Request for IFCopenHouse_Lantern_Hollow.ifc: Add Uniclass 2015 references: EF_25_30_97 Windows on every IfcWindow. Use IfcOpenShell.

First a look at what the model holds.

```python
import ifcopenshell

model = ifcopenshell.open("IFCopenHouse_Lantern_Hollow.ifc")
print(model.schema)
print("classifications:", [c.Name for c in model.by_type("IfcClassification")])
for ifc_class in ("IfcDoor", "IfcRoof", "IfcStair", "IfcWall", "IfcWindow"):
    print(ifc_class, len(model.by_type(ifc_class)))
```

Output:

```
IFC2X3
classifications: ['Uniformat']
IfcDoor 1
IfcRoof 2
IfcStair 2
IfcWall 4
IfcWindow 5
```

```python
import ifcopenshell
import ifcopenshell.api.classification

model = ifcopenshell.open("IFCopenHouse_Lantern_Hollow.ifc")

# IFC2X3 requires Source and Edition and has no link from the project to the system.
system = model.create_entity("IfcClassification", Source="NBS", Edition="2015", Name="Uniclass 2015")

codes = {
    "IfcWindow": ("EF_25_30_97", "Windows"),
}
for ifc_class, (code, name) in codes.items():
    products = model.by_type(ifc_class)
    ifcopenshell.api.classification.add_reference(
        model, products=products, classification=system, identification=code, name=name
    )
    print(code, len(products))

model.write("IFCopenHouse_Lantern_Hollow_v2.ifc")
```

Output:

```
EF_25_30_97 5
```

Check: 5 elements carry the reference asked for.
